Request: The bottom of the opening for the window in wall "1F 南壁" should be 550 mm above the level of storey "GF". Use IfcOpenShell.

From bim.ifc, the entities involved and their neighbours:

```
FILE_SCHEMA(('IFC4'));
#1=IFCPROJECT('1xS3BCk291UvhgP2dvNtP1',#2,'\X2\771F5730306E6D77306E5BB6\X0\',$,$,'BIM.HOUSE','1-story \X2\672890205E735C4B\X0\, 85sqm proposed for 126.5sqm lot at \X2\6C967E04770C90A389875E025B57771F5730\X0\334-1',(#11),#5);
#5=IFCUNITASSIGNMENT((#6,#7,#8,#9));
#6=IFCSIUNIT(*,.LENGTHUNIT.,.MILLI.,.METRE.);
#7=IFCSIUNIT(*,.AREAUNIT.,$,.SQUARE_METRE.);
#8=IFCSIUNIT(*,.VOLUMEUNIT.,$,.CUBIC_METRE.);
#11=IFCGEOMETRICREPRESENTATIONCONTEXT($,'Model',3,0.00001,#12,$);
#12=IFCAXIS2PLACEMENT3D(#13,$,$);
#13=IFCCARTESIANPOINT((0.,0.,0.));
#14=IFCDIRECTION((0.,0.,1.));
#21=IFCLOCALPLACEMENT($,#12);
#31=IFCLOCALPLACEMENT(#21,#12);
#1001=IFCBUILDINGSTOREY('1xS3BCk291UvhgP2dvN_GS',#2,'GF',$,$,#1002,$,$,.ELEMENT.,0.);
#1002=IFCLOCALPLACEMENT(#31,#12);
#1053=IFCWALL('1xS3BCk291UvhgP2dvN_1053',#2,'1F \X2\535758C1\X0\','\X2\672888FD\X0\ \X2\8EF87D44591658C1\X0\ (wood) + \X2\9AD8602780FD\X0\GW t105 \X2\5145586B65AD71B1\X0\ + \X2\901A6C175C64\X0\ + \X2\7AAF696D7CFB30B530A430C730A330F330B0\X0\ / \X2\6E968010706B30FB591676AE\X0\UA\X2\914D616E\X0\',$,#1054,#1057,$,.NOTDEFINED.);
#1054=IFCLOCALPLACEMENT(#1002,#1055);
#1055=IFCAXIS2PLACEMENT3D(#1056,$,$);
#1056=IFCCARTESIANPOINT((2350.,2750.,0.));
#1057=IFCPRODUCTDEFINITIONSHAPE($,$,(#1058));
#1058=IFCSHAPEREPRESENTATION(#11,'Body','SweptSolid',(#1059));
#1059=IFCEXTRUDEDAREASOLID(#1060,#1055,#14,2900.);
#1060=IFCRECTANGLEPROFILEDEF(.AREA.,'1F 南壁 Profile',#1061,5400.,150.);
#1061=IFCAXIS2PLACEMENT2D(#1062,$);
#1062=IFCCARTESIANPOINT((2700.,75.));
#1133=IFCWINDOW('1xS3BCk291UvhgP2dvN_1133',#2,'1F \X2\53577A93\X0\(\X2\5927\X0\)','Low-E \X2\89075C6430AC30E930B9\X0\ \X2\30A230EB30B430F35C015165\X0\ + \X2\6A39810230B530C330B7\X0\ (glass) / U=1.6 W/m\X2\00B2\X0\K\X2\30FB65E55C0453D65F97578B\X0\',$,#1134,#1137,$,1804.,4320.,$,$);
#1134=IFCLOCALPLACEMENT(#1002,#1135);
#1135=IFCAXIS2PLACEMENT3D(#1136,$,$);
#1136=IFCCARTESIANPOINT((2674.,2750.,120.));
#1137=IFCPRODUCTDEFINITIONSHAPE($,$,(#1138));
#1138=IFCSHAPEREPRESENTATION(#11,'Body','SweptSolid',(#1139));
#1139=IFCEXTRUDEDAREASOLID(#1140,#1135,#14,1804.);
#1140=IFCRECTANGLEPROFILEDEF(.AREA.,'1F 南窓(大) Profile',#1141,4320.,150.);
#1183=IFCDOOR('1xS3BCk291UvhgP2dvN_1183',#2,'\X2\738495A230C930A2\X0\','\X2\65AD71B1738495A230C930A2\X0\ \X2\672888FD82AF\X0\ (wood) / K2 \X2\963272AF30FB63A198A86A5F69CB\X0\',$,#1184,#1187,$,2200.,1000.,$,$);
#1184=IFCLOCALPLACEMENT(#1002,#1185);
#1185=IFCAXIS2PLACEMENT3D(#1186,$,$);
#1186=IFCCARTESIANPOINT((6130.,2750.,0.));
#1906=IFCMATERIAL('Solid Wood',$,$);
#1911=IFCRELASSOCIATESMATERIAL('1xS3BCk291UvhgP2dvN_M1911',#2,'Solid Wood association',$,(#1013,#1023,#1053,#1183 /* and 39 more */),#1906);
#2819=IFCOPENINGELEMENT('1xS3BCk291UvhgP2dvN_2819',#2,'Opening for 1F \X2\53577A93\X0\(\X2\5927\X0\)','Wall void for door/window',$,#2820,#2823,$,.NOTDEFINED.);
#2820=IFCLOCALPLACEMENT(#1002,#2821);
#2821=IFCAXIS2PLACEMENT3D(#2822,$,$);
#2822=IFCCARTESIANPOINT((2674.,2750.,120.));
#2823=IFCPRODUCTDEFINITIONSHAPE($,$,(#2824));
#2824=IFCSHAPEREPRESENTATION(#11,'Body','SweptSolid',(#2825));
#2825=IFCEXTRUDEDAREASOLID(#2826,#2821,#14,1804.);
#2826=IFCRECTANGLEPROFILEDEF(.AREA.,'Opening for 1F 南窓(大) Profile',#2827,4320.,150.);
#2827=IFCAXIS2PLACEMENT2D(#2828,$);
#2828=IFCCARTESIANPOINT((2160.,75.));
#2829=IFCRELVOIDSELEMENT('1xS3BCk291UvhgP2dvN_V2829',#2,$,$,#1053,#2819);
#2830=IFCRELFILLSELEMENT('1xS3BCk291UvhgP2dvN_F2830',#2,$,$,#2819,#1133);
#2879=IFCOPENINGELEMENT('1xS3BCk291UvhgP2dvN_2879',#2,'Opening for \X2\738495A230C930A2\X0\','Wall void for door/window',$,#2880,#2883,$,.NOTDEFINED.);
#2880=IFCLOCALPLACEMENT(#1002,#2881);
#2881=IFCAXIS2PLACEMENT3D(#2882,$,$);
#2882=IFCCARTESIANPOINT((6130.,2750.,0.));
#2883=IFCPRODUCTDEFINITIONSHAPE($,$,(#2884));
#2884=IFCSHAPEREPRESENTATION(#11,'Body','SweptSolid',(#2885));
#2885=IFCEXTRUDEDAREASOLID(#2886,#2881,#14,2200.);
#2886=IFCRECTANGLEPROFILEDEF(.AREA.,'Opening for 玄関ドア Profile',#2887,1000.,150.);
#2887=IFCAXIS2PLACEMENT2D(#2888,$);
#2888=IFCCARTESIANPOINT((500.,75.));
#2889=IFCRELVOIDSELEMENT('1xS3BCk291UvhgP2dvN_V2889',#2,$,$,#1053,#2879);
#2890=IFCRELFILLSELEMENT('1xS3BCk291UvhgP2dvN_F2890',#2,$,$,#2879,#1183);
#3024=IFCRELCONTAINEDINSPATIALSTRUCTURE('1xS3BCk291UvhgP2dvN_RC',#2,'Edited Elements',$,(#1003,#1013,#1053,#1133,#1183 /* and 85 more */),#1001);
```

```python
import numpy as np
import ifcopenshell
import ifcopenshell.api.geometry
import ifcopenshell.geom
import ifcopenshell.util.element
import ifcopenshell.util.placement
import ifcopenshell.util.shape
import ifcopenshell.util.unit

model = ifcopenshell.open("bim.ifc")
unit_scale = ifcopenshell.util.unit.calculate_unit_scale(model)

window = model.by_guid("1xS3BCk291UvhgP2dvN_1133")
opening = window.FillsVoids[0].RelatingOpeningElement
storey = ifcopenshell.util.element.get_container(window, ifc_class="IfcBuildingStorey")
level = ifcopenshell.util.placement.get_local_placement(storey.ObjectPlacement)[2, 3]

# The opening's origin need not be at the sill, so measure its lowest point.
shape = ifcopenshell.geom.create_shape(ifcopenshell.geom.settings(), opening)
bottom = ifcopenshell.util.shape.get_shape_bottom_elevation(shape, shape.geometry) / unit_scale
dz = level + 0.55 / unit_scale - bottom

shift = np.array([0.0, 0.0, dz])
# The window is not placed relative to its opening, so move both.
for product in (opening, window):
    matrix = ifcopenshell.util.placement.get_local_placement(product.ObjectPlacement)
    matrix[:3, 3] += shift
    ifcopenshell.api.geometry.edit_object_placement(model, product=product, matrix=matrix, is_si=False)

print(f"moved by {dz * unit_scale:+.3f} m")

model.write("bim_edited.ifc")
```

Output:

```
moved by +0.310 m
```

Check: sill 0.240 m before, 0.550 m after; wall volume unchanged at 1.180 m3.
